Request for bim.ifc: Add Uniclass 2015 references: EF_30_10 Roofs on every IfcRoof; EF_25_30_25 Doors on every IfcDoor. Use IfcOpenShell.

First a look at what the model holds.

```python
import ifcopenshell

model = ifcopenshell.open("bim.ifc")
print(model.schema)
print("classifications:", [c.Name for c in model.by_type("IfcClassification")])
for ifc_class in ("IfcDoor", "IfcRoof", "IfcStair", "IfcWall", "IfcWindow"):
    print(ifc_class, len(model.by_type(ifc_class)))
```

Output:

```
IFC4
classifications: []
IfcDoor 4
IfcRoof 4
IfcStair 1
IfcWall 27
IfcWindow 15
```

```python
import ifcopenshell
import ifcopenshell.api.classification

model = ifcopenshell.open("bim.ifc")

system = ifcopenshell.api.classification.add_classification(model, classification="Uniclass 2015")

codes = {
    "IfcRoof": ("EF_30_10", "Roofs"),
    "IfcDoor": ("EF_25_30_25", "Doors"),
}
for ifc_class, (code, name) in codes.items():
    products = model.by_type(ifc_class)
    ifcopenshell.api.classification.add_reference(
        model, products=products, classification=system, identification=code, name=name
    )
    print(code, len(products))

model.write("bim-out.ifc")
```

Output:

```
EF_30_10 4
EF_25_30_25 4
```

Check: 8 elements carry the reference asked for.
